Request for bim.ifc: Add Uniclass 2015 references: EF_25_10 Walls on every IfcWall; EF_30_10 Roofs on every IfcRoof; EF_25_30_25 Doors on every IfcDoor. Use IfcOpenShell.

First a look at what the model holds.

```python
import ifcopenshell

model = ifcopenshell.open("bim.ifc")
print(model.schema)
print("classifications:", [c.Name for c in model.by_type("IfcClassification")])
for ifc_class in ("IfcDoor", "IfcRoof", "IfcStair", "IfcWall", "IfcWindow"):
    print(ifc_class, len(model.by_type(ifc_class)))
```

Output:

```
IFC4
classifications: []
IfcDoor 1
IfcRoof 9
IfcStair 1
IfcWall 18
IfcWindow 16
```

```python
import ifcopenshell
import ifcopenshell.api.classification

model = ifcopenshell.open("bim.ifc")

system = ifcopenshell.api.classification.add_classification(model, classification="Uniclass 2015")

codes = {
    "IfcWall": ("EF_25_10", "Walls"),
    "IfcRoof": ("EF_30_10", "Roofs"),
    "IfcDoor": ("EF_25_30_25", "Doors"),
}
for ifc_class, (code, name) in codes.items():
    products = model.by_type(ifc_class)
    ifcopenshell.api.classification.add_reference(
        model, products=products, classification=system, identification=code, name=name
    )
    print(code, len(products))

model.write("bim_rev.ifc")
```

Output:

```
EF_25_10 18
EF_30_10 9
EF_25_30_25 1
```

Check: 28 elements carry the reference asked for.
